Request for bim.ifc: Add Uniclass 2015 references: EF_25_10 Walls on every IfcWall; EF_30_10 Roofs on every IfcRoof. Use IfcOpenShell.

First a look at what the model holds.

```python
import ifcopenshell

model = ifcopenshell.open("bim.ifc")
print(model.schema)
print("classifications:", [c.Name for c in model.by_type("IfcClassification")])
for ifc_class in ("IfcDoor", "IfcRoof", "IfcStair", "IfcWall", "IfcWindow"):
    print(ifc_class, len(model.by_type(ifc_class)))
```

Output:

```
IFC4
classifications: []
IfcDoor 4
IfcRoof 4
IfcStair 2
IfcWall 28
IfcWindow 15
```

```python
import ifcopenshell
import ifcopenshell.api.classification

model = ifcopenshell.open("bim.ifc")

system = ifcopenshell.api.classification.add_classification(model, classification="Uniclass 2015")

codes = {
    "IfcWall": ("EF_25_10", "Walls"),
    "IfcRoof": ("EF_30_10", "Roofs"),
}
for ifc_class, (code, name) in codes.items():
    products = model.by_type(ifc_class)
    ifcopenshell.api.classification.add_reference(
        model, products=products, classification=system, identification=code, name=name
    )
    print(code, len(products))

model.write("bim-out.ifc")
```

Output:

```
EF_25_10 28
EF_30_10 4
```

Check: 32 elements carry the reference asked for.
